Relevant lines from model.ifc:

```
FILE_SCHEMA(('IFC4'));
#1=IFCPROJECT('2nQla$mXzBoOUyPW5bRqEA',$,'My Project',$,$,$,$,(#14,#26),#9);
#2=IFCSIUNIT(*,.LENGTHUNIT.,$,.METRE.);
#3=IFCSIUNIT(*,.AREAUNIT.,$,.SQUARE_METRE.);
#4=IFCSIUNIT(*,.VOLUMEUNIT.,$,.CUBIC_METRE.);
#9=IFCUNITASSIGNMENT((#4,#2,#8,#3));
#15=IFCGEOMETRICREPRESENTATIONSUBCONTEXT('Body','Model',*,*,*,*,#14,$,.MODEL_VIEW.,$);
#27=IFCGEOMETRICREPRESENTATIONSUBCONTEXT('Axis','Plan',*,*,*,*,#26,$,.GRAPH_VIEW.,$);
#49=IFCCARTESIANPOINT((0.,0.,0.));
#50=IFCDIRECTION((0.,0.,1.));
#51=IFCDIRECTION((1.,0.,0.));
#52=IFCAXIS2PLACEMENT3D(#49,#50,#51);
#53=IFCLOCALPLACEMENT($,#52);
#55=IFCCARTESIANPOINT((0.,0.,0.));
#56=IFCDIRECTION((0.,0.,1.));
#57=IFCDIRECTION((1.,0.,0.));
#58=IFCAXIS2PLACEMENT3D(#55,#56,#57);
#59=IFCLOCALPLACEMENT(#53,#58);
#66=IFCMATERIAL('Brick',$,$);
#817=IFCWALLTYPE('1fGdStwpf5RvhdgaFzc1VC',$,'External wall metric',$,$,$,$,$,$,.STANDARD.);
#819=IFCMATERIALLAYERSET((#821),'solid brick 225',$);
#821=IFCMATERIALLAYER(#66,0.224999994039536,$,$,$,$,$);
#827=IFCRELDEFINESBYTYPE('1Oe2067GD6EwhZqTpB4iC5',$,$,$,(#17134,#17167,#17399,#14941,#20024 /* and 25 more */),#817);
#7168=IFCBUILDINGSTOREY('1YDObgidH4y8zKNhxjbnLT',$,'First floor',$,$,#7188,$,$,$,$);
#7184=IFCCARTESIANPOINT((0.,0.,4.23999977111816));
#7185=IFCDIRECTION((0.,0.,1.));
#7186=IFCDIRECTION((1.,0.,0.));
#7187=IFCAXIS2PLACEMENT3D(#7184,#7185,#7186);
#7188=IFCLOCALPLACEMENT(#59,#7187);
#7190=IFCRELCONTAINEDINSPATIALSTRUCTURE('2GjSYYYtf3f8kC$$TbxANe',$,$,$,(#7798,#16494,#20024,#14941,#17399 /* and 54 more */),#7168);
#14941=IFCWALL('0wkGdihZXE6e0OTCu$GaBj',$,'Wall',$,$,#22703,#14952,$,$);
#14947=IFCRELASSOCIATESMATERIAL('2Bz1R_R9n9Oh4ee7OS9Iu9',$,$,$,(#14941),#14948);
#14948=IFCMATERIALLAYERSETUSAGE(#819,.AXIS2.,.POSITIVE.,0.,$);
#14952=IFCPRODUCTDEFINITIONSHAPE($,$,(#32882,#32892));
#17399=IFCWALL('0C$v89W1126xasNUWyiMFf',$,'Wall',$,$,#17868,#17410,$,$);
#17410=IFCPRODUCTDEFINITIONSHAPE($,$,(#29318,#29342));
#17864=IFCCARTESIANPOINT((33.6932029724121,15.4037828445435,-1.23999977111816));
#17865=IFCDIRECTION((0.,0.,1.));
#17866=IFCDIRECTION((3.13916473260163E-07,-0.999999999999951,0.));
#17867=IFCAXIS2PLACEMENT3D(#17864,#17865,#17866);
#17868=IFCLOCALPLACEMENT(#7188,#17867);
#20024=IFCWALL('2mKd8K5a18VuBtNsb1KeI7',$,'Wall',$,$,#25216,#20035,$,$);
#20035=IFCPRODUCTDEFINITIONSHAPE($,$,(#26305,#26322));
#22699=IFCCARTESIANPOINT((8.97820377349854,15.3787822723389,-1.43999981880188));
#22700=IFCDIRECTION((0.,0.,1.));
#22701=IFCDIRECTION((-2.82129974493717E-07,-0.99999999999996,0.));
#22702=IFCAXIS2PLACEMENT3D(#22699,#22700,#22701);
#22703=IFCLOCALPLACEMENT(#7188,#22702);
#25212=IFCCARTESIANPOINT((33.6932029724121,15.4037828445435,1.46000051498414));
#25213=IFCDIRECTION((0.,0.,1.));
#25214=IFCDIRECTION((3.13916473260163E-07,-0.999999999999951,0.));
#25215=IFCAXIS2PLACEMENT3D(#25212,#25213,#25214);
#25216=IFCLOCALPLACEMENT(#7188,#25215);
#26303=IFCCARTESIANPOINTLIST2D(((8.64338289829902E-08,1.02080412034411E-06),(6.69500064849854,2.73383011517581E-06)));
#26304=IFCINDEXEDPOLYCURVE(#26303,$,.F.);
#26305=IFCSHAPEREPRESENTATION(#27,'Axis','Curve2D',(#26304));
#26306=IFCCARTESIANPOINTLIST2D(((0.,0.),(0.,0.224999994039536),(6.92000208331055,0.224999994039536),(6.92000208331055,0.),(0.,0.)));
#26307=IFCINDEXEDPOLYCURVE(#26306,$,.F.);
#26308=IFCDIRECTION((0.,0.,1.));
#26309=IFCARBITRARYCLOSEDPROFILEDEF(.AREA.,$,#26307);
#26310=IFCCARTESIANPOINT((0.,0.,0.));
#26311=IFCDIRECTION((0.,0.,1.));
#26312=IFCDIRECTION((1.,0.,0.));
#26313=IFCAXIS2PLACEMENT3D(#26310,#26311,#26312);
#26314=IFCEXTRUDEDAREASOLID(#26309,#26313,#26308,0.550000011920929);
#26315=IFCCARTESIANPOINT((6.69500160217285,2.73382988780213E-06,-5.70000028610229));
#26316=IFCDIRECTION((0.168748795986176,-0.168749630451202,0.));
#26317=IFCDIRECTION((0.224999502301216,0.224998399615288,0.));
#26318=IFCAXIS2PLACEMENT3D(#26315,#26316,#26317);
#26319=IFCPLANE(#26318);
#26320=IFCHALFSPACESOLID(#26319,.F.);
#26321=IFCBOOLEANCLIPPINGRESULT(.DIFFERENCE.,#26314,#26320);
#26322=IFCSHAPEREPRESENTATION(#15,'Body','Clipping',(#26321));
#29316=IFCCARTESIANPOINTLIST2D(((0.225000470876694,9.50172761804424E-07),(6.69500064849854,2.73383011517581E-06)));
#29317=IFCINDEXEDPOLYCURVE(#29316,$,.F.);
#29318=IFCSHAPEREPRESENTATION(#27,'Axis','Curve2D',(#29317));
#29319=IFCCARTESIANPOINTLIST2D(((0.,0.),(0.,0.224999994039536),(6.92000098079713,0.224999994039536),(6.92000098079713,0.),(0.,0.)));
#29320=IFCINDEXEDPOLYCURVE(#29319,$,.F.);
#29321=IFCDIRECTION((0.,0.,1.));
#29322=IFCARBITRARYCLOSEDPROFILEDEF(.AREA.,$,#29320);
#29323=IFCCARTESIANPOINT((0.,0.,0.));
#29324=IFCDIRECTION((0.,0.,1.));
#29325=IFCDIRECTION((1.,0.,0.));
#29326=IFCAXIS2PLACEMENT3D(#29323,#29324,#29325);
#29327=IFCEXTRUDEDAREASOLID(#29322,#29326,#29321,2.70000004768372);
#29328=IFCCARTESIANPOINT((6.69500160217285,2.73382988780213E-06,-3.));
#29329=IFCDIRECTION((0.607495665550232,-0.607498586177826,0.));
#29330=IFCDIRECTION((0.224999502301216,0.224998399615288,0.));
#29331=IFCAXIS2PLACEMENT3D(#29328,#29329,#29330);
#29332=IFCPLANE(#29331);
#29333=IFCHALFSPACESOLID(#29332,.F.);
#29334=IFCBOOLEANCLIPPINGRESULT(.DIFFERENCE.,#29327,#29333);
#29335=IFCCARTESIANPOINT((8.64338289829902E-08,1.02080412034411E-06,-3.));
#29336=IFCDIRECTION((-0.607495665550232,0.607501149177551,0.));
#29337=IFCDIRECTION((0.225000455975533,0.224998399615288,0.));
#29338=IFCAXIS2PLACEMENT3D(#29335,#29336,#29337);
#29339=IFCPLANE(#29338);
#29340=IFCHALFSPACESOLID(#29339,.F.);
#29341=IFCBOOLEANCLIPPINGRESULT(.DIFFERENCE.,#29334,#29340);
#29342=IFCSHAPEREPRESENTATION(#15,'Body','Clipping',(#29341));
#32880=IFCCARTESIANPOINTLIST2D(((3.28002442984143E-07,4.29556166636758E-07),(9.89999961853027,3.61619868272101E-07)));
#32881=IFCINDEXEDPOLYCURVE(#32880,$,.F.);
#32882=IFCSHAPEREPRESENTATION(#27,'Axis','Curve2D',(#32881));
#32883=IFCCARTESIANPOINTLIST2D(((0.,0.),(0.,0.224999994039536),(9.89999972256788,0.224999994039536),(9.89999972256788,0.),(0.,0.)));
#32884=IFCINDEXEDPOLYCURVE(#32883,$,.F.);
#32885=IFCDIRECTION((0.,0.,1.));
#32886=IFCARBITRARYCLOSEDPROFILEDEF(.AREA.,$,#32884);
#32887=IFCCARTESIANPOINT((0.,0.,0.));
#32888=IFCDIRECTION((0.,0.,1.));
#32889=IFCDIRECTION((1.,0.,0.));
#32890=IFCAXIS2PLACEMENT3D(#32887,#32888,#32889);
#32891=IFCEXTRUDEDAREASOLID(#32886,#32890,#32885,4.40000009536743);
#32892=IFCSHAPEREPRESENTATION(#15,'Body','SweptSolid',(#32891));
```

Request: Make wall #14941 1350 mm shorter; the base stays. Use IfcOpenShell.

```python
import ifcopenshell
import ifcopenshell.geom
import ifcopenshell.util.representation
import ifcopenshell.util.shape
import ifcopenshell.util.unit

model = ifcopenshell.open("model.ifc")
unit_scale = ifcopenshell.util.unit.calculate_unit_scale(model)
settings = ifcopenshell.geom.settings()


def volume(element):
    """Net volume in cubic metres, openings subtracted."""
    shape = ifcopenshell.geom.create_shape(settings, element)
    return ifcopenshell.util.shape.get_volume(shape.geometry)


wall = model.by_guid("0wkGdihZXE6e0OTCu$GaBj")
before = volume(wall)

body = ifcopenshell.util.representation.get_representation(wall, "Model", "Body")
solid = body.Items[0]
old_height = solid.Depth
solid.Depth -= 1.35 / unit_scale
after = volume(wall)

print(f"height {old_height:g} -> {solid.Depth:g}, volume {before:.3f} -> {after:.3f} m3")

model.write("model_rev.ifc")
```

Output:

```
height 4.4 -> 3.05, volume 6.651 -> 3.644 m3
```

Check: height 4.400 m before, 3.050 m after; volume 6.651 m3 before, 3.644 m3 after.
